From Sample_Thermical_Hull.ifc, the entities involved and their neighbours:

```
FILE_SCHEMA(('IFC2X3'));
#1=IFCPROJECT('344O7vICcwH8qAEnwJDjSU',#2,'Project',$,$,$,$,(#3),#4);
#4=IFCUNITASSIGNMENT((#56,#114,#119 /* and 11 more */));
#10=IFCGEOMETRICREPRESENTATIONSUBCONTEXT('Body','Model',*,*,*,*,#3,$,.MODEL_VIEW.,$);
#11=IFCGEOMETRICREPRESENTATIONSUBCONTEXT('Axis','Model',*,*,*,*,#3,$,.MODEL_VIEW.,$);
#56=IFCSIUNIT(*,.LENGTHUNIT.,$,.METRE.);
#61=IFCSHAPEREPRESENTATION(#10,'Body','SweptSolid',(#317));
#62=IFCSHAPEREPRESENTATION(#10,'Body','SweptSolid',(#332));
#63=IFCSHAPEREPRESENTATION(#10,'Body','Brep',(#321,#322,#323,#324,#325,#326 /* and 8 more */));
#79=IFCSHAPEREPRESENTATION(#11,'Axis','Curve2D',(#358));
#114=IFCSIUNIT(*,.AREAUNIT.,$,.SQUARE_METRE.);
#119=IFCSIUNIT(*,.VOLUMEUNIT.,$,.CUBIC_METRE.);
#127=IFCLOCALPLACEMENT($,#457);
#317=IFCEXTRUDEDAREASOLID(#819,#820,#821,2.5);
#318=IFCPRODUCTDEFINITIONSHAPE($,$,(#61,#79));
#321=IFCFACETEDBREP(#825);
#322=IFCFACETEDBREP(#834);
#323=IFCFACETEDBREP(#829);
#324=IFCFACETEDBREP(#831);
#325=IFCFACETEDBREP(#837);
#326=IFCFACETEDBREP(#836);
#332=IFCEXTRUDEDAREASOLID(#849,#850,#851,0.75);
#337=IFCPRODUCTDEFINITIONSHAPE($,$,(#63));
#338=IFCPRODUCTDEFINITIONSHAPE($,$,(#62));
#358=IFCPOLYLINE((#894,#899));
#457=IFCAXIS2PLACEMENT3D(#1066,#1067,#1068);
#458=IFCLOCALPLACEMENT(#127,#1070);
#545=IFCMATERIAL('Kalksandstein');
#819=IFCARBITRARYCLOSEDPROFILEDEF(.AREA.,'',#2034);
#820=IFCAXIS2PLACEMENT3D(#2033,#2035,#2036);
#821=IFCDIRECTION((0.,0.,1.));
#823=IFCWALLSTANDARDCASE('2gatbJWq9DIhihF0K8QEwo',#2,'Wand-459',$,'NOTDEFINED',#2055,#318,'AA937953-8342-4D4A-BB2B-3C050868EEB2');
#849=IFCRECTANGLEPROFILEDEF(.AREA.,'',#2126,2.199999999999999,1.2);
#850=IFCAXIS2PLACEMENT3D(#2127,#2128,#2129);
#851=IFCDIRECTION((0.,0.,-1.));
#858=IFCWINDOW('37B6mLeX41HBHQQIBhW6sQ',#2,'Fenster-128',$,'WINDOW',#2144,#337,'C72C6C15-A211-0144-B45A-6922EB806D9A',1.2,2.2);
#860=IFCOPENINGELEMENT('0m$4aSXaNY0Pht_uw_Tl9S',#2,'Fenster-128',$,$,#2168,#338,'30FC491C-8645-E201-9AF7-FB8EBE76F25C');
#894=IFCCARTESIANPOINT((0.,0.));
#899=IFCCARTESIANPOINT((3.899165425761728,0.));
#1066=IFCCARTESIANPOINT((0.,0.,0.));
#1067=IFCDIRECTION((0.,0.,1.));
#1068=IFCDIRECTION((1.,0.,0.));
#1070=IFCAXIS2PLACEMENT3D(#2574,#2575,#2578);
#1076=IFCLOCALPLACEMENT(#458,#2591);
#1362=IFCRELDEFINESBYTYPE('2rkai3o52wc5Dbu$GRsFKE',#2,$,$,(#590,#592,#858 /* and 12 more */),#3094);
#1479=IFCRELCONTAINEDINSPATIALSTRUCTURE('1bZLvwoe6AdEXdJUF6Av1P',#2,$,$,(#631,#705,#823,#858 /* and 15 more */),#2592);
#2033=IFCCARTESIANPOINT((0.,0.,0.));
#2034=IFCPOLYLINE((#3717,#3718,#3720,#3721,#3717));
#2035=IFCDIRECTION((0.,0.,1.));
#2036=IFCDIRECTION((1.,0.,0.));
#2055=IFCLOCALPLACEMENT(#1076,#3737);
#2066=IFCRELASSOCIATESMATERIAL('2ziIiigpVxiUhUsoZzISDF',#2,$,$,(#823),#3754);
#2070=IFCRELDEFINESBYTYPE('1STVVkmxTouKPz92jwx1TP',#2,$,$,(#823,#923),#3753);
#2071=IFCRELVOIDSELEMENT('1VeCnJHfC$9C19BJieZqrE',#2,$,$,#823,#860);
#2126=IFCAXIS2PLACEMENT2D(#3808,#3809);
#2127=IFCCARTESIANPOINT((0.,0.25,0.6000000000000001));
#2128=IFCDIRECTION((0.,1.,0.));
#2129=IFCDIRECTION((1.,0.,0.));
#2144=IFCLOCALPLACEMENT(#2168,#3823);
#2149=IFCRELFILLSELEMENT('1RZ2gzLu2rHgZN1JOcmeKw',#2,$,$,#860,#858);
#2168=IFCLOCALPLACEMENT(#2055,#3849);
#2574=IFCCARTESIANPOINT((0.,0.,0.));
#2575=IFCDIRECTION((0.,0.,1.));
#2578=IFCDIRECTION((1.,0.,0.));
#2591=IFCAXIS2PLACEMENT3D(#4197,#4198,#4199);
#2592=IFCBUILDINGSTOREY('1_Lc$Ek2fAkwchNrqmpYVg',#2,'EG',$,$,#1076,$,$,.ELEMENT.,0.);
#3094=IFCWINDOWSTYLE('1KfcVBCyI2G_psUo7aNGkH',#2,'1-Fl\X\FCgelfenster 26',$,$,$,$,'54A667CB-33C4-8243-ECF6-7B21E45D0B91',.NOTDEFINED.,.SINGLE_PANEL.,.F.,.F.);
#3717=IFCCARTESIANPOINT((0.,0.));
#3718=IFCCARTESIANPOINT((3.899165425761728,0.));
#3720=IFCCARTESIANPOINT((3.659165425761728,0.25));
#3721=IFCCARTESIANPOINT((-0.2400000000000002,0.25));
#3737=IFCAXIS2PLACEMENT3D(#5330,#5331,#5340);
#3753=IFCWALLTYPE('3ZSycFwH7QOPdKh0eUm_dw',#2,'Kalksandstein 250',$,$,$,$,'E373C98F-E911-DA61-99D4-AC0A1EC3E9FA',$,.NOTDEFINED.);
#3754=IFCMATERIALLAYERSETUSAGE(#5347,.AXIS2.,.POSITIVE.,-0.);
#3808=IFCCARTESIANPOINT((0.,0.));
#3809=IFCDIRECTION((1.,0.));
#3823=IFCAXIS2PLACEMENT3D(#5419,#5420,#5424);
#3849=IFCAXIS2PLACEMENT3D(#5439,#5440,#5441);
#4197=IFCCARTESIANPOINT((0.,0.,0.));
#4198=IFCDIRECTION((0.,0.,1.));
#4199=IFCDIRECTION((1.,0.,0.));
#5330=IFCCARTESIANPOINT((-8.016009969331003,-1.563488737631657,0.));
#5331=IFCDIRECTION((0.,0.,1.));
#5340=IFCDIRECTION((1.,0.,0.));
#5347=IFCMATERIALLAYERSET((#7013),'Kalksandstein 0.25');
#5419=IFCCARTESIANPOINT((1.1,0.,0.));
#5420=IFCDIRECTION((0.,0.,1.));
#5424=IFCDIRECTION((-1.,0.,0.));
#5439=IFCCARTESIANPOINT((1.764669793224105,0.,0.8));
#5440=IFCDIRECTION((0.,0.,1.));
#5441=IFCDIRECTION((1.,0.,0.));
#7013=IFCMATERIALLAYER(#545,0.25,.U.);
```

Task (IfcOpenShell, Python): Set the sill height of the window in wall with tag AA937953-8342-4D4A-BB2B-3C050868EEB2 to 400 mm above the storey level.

```python
import numpy as np
import ifcopenshell
import ifcopenshell.api.geometry
import ifcopenshell.geom
import ifcopenshell.util.element
import ifcopenshell.util.placement
import ifcopenshell.util.shape
import ifcopenshell.util.unit

model = ifcopenshell.open("Sample_Thermical_Hull.ifc")
unit_scale = ifcopenshell.util.unit.calculate_unit_scale(model)

window = model.by_guid("37B6mLeX41HBHQQIBhW6sQ")
opening = window.FillsVoids[0].RelatingOpeningElement
storey = ifcopenshell.util.element.get_container(window, ifc_class="IfcBuildingStorey")
level = ifcopenshell.util.placement.get_local_placement(storey.ObjectPlacement)[2, 3]

# The opening's origin need not be at the sill, so measure its lowest point.
shape = ifcopenshell.geom.create_shape(ifcopenshell.geom.settings(), opening)
bottom = ifcopenshell.util.shape.get_shape_bottom_elevation(shape, shape.geometry) / unit_scale
dz = level + 0.4 / unit_scale - bottom

shift = np.array([0.0, 0.0, dz])
# The window is placed relative to its opening, so it follows when the opening moves.
matrix = ifcopenshell.util.placement.get_local_placement(opening.ObjectPlacement)
matrix[:3, 3] += shift
ifcopenshell.api.geometry.edit_object_placement(
    model, product=opening, matrix=matrix, is_si=False, should_transform_children=True
)

print(f"moved by {dz * unit_scale:+.3f} m")

model.write("Sample_Thermical_Hull_edited.ifc")
```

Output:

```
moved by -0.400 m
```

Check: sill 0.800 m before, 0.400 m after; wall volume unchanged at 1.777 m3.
